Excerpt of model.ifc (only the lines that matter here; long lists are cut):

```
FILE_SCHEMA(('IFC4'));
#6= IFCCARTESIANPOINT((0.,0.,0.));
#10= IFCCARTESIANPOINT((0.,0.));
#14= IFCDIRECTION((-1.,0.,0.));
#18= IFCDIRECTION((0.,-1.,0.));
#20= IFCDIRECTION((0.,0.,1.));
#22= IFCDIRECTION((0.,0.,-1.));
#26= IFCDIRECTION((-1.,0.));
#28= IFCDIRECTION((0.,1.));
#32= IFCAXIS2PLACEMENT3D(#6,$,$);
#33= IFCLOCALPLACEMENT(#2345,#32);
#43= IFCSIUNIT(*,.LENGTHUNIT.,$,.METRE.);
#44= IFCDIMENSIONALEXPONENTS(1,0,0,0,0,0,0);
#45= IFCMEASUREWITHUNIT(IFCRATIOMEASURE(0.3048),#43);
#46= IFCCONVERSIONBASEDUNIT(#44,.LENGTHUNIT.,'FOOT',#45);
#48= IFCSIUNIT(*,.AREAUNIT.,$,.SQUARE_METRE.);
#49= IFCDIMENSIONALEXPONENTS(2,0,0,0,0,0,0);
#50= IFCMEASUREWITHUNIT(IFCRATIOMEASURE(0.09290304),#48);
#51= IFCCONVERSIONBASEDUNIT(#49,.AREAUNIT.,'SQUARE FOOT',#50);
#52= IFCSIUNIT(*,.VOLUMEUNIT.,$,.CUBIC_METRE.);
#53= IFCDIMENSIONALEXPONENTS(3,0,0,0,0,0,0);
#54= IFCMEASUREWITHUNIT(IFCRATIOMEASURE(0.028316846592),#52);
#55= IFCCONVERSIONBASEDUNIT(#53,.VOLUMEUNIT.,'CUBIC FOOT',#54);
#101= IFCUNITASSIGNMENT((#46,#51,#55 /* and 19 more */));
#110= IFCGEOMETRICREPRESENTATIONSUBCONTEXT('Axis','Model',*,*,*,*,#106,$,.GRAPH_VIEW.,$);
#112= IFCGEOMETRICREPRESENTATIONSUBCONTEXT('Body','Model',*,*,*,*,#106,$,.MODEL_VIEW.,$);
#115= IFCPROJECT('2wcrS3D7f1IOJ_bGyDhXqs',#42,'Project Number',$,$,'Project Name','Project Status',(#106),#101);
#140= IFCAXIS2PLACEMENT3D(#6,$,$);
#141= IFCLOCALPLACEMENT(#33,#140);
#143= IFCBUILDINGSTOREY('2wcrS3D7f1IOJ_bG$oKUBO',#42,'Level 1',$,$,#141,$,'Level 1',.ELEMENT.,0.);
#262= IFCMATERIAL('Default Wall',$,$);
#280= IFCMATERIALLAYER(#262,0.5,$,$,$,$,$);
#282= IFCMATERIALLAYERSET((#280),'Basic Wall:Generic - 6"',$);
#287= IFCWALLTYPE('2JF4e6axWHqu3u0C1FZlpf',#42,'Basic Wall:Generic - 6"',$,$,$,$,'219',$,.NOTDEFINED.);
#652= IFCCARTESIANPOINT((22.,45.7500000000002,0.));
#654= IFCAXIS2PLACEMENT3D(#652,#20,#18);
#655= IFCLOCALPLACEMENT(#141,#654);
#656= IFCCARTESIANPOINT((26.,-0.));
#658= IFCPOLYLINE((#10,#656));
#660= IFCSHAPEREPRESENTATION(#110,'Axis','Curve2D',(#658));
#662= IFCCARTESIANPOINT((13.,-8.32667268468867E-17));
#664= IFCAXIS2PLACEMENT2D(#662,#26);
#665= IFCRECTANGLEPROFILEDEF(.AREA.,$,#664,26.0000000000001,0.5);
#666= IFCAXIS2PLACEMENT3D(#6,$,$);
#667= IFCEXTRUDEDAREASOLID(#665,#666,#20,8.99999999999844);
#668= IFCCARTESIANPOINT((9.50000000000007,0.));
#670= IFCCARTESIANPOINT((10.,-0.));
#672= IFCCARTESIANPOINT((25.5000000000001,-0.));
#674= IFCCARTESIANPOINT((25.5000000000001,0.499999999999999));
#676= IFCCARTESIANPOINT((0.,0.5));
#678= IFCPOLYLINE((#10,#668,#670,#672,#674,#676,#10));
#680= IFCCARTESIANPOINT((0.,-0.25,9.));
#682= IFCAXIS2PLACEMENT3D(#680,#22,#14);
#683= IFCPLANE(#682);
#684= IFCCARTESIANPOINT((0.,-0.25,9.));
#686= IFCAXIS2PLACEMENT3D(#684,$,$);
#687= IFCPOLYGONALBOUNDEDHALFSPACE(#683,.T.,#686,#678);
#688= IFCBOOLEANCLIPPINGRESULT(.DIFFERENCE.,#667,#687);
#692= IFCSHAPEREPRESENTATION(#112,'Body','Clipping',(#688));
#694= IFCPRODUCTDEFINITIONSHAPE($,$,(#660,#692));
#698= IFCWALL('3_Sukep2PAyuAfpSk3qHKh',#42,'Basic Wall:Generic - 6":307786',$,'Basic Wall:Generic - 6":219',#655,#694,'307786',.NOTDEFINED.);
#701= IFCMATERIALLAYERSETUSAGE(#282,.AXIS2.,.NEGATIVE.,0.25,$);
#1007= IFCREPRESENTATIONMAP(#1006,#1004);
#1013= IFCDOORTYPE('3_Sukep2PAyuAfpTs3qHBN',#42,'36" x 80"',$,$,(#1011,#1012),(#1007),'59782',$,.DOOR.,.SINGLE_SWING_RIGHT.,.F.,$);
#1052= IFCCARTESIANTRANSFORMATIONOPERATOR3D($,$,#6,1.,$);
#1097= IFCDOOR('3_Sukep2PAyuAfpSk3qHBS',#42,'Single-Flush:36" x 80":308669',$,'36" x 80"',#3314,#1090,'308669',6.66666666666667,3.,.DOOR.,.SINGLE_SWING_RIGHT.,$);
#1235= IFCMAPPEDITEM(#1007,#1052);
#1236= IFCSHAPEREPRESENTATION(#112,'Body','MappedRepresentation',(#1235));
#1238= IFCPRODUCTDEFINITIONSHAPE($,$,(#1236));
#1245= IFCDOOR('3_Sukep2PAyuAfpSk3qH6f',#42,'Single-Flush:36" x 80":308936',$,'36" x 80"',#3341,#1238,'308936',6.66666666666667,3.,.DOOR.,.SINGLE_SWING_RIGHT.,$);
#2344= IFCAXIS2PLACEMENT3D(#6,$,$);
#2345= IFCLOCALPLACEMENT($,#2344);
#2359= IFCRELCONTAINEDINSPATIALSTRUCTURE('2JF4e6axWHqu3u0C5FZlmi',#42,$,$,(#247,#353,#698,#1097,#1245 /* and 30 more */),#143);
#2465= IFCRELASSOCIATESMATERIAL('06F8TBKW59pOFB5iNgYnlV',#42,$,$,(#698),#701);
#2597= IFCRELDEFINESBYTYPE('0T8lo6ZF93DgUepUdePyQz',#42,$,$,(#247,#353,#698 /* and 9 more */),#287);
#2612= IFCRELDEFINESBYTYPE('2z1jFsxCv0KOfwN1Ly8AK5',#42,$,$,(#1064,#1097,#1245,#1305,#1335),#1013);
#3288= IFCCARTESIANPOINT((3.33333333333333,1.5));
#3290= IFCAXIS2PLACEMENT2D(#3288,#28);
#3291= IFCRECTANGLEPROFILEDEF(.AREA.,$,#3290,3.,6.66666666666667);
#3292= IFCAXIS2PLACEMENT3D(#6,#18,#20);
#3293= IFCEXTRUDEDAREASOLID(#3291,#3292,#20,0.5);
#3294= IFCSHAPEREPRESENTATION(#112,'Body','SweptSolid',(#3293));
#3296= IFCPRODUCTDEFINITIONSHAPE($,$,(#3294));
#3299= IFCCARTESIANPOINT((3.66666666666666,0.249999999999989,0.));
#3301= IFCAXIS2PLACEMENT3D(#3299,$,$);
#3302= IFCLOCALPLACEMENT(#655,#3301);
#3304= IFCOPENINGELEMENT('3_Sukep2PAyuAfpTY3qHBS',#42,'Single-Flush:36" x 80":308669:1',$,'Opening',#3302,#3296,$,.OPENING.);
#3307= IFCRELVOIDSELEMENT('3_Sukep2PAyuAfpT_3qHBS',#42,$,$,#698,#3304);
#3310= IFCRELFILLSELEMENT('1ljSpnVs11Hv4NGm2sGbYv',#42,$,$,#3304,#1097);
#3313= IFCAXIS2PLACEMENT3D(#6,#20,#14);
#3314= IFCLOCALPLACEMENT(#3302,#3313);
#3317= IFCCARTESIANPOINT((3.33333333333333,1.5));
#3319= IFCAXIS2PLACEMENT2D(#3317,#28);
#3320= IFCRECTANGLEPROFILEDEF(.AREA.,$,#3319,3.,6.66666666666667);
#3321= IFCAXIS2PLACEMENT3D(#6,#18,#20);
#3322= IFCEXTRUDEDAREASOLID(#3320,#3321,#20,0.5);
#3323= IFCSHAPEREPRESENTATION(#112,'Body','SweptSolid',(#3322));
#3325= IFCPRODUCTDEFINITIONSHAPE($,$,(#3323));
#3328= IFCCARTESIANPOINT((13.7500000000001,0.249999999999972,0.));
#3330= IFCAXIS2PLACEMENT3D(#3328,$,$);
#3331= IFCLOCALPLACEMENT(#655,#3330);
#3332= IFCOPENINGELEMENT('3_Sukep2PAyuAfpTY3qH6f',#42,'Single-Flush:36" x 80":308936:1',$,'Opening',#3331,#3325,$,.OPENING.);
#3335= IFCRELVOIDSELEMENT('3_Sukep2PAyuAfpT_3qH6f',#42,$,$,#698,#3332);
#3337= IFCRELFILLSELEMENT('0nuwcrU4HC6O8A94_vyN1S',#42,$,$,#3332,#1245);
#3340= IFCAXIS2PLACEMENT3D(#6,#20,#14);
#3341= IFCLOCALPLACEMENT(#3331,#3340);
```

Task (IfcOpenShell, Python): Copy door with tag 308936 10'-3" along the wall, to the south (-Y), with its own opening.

```python
import ifcopenshell
import ifcopenshell.api.feature
import ifcopenshell.api.geometry
import ifcopenshell.api.root
import ifcopenshell.geom
import ifcopenshell.util.element
import ifcopenshell.util.placement
import ifcopenshell.util.shape
import ifcopenshell.util.unit

model = ifcopenshell.open("model.ifc")
unit_scale = ifcopenshell.util.unit.calculate_unit_scale(model)
settings = ifcopenshell.geom.settings()


def volume(element):
    """Net volume in cubic metres, openings subtracted."""
    shape = ifcopenshell.geom.create_shape(settings, element)
    return ifcopenshell.util.shape.get_volume(shape.geometry)


def reuse_history(source, copy):
    """copy_class also copies each property set's owner history, people and application; keep the originals."""
    for rel in copy.IsDefinedBy:
        if rel.is_a("IfcRelDefinesByProperties") and (history := rel.RelatingPropertyDefinition.OwnerHistory):
            rel.RelatingPropertyDefinition.OwnerHistory = source.OwnerHistory
            ifcopenshell.util.element.remove_deep2(model, history)


door = model.by_guid("3_Sukep2PAyuAfpSk3qH6f")
opening = door.FillsVoids[0].RelatingOpeningElement
wall = opening.VoidsElements[0].RelatingBuildingElement
before = volume(wall)
shift = ifcopenshell.util.placement.get_local_placement(wall.ObjectPlacement)[:3, 0] * 123 * 0.0254 / unit_scale

# copy_class copies the void relationship, type, container and properties, but no geometry.
new_opening = ifcopenshell.api.root.copy_class(model, product=opening)
new_opening.Representation = ifcopenshell.util.element.copy_deep(
    model, opening.Representation, exclude=["IfcGeometricRepresentationContext", "IfcRepresentationMap"]
)
new_opening.Name = 'Single-Flush:36" x 80"'
new_door = ifcopenshell.api.root.copy_class(model, product=door)
new_door.Representation = ifcopenshell.util.element.copy_deep(
    model, door.Representation, exclude=["IfcGeometricRepresentationContext", "IfcRepresentationMap"]
)
new_door.Name = 'Single-Flush:36" x 80"'
new_door.Tag = None
reuse_history(door, new_door)
ifcopenshell.api.feature.add_filling(model, opening=new_opening, element=new_door)

for old, new in ((opening, new_opening), (door, new_door)):
    matrix = ifcopenshell.util.placement.get_local_placement(old.ObjectPlacement)
    matrix[:3, 3] += shift
    ifcopenshell.api.geometry.edit_object_placement(model, product=new, matrix=matrix, is_si=False)

after = volume(wall)

print(f"wall volume {before:.3f} -> {after:.3f} m3")

model.write("model_edited.ifc")
```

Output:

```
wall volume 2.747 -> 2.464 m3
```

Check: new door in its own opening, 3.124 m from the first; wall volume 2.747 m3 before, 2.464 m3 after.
